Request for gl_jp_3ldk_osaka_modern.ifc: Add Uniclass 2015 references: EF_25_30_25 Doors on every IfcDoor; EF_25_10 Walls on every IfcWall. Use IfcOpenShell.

First a look at what the model holds.

```python
import ifcopenshell

model = ifcopenshell.open("gl_jp_3ldk_osaka_modern.ifc")
print(model.schema)
print("classifications:", [c.Name for c in model.by_type("IfcClassification")])
for ifc_class in ("IfcDoor", "IfcRoof", "IfcStair", "IfcWall", "IfcWindow"):
    print(ifc_class, len(model.by_type(ifc_class)))
```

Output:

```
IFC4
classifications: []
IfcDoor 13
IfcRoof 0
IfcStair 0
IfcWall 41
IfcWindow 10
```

```python
import ifcopenshell
import ifcopenshell.api.classification

model = ifcopenshell.open("gl_jp_3ldk_osaka_modern.ifc")

system = ifcopenshell.api.classification.add_classification(model, classification="Uniclass 2015")

codes = {
    "IfcDoor": ("EF_25_30_25", "Doors"),
    "IfcWall": ("EF_25_10", "Walls"),
}
for ifc_class, (code, name) in codes.items():
    products = model.by_type(ifc_class)
    ifcopenshell.api.classification.add_reference(
        model, products=products, classification=system, identification=code, name=name
    )
    print(code, len(products))

model.write("gl_jp_3ldk_osaka_modern_rev.ifc")
```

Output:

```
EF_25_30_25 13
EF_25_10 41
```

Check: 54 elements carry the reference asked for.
